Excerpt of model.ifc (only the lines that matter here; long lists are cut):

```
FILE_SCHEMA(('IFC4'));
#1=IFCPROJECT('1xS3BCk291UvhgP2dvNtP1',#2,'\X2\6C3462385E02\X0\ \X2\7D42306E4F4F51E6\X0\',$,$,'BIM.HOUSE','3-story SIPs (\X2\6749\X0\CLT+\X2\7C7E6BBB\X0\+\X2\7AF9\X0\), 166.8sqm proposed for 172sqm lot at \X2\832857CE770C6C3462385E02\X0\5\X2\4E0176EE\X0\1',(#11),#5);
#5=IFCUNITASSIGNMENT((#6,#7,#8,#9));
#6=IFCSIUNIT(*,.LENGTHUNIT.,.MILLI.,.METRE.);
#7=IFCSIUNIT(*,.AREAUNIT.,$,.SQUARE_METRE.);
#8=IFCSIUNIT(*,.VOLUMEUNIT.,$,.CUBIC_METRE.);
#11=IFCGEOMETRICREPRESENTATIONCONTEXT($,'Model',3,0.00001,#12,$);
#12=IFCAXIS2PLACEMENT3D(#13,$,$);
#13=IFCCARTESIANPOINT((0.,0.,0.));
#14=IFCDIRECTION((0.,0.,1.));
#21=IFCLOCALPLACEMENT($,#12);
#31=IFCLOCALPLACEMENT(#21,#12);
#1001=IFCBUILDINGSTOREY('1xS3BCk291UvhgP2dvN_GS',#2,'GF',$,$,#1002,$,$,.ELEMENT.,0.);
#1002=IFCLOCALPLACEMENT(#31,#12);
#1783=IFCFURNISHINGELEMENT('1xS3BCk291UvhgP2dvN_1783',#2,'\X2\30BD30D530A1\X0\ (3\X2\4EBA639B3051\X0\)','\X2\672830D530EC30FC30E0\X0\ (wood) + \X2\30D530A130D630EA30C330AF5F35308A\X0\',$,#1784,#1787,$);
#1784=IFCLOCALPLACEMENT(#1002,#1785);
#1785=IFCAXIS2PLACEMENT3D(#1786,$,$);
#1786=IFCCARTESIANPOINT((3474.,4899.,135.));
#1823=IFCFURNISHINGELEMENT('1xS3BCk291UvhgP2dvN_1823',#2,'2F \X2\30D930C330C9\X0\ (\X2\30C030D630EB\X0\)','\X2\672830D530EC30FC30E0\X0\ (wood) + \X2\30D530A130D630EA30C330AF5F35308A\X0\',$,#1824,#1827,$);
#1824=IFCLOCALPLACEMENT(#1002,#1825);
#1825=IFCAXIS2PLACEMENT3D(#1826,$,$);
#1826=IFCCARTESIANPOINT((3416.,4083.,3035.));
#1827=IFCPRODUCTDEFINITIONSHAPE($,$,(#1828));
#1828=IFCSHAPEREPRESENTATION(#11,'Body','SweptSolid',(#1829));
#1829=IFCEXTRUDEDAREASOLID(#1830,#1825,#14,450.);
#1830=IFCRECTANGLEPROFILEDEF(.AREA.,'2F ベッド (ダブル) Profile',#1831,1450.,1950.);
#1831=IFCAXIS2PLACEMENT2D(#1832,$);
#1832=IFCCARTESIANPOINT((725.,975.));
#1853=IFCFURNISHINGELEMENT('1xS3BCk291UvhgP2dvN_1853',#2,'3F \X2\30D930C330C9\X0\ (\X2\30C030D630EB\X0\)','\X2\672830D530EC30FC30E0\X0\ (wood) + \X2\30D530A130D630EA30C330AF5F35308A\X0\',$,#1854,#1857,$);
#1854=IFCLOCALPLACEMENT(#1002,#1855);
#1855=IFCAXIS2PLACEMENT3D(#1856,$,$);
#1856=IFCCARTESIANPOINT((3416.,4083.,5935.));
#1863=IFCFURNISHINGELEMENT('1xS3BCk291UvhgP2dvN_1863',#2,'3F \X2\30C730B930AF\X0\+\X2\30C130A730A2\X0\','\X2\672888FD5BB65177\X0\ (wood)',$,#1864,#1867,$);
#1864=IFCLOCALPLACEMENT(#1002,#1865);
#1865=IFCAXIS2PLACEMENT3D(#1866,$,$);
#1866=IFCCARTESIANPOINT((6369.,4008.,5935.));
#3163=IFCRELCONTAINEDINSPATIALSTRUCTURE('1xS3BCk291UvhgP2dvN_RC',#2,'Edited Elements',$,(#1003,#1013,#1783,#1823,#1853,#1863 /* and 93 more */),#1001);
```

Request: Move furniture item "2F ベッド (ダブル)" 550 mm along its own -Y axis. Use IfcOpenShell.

```python
import ifcopenshell
import ifcopenshell.api.geometry
import ifcopenshell.util.placement
import ifcopenshell.util.unit

model = ifcopenshell.open("model.ifc")
unit_scale = ifcopenshell.util.unit.calculate_unit_scale(model)

item = model.by_guid("1xS3BCk291UvhgP2dvN_1823")
matrix = ifcopenshell.util.placement.get_local_placement(item.ObjectPlacement)
matrix[:3, 3] -= matrix[:3, 1] * 0.55 / unit_scale
ifcopenshell.api.geometry.edit_object_placement(model, product=item, matrix=matrix, is_si=False)

print(ifcopenshell.util.placement.get_local_placement(item.ObjectPlacement).round(3) + 0.0)

model.write("model_rev.ifc")
```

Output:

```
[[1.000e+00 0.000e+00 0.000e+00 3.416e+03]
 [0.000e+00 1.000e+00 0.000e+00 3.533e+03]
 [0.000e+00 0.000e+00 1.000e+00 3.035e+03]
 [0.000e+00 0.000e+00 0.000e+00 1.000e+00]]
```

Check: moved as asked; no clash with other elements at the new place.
